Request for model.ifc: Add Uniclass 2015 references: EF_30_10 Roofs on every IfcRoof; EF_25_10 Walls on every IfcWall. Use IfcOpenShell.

First a look at what the model holds.

```python
import ifcopenshell

model = ifcopenshell.open("model.ifc")
print(model.schema)
print("classifications:", [c.Name for c in model.by_type("IfcClassification")])
for ifc_class in ("IfcDoor", "IfcRoof", "IfcStair", "IfcWall", "IfcWindow"):
    print(ifc_class, len(model.by_type(ifc_class)))
```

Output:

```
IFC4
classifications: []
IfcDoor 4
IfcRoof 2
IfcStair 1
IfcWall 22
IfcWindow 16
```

```python
import ifcopenshell
import ifcopenshell.api.classification

model = ifcopenshell.open("model.ifc")

system = ifcopenshell.api.classification.add_classification(model, classification="Uniclass 2015")

codes = {
    "IfcRoof": ("EF_30_10", "Roofs"),
    "IfcWall": ("EF_25_10", "Walls"),
}
for ifc_class, (code, name) in codes.items():
    products = model.by_type(ifc_class)
    ifcopenshell.api.classification.add_reference(
        model, products=products, classification=system, identification=code, name=name
    )
    print(code, len(products))

model.write("model_v2.ifc")
```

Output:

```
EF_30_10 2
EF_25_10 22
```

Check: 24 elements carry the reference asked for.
